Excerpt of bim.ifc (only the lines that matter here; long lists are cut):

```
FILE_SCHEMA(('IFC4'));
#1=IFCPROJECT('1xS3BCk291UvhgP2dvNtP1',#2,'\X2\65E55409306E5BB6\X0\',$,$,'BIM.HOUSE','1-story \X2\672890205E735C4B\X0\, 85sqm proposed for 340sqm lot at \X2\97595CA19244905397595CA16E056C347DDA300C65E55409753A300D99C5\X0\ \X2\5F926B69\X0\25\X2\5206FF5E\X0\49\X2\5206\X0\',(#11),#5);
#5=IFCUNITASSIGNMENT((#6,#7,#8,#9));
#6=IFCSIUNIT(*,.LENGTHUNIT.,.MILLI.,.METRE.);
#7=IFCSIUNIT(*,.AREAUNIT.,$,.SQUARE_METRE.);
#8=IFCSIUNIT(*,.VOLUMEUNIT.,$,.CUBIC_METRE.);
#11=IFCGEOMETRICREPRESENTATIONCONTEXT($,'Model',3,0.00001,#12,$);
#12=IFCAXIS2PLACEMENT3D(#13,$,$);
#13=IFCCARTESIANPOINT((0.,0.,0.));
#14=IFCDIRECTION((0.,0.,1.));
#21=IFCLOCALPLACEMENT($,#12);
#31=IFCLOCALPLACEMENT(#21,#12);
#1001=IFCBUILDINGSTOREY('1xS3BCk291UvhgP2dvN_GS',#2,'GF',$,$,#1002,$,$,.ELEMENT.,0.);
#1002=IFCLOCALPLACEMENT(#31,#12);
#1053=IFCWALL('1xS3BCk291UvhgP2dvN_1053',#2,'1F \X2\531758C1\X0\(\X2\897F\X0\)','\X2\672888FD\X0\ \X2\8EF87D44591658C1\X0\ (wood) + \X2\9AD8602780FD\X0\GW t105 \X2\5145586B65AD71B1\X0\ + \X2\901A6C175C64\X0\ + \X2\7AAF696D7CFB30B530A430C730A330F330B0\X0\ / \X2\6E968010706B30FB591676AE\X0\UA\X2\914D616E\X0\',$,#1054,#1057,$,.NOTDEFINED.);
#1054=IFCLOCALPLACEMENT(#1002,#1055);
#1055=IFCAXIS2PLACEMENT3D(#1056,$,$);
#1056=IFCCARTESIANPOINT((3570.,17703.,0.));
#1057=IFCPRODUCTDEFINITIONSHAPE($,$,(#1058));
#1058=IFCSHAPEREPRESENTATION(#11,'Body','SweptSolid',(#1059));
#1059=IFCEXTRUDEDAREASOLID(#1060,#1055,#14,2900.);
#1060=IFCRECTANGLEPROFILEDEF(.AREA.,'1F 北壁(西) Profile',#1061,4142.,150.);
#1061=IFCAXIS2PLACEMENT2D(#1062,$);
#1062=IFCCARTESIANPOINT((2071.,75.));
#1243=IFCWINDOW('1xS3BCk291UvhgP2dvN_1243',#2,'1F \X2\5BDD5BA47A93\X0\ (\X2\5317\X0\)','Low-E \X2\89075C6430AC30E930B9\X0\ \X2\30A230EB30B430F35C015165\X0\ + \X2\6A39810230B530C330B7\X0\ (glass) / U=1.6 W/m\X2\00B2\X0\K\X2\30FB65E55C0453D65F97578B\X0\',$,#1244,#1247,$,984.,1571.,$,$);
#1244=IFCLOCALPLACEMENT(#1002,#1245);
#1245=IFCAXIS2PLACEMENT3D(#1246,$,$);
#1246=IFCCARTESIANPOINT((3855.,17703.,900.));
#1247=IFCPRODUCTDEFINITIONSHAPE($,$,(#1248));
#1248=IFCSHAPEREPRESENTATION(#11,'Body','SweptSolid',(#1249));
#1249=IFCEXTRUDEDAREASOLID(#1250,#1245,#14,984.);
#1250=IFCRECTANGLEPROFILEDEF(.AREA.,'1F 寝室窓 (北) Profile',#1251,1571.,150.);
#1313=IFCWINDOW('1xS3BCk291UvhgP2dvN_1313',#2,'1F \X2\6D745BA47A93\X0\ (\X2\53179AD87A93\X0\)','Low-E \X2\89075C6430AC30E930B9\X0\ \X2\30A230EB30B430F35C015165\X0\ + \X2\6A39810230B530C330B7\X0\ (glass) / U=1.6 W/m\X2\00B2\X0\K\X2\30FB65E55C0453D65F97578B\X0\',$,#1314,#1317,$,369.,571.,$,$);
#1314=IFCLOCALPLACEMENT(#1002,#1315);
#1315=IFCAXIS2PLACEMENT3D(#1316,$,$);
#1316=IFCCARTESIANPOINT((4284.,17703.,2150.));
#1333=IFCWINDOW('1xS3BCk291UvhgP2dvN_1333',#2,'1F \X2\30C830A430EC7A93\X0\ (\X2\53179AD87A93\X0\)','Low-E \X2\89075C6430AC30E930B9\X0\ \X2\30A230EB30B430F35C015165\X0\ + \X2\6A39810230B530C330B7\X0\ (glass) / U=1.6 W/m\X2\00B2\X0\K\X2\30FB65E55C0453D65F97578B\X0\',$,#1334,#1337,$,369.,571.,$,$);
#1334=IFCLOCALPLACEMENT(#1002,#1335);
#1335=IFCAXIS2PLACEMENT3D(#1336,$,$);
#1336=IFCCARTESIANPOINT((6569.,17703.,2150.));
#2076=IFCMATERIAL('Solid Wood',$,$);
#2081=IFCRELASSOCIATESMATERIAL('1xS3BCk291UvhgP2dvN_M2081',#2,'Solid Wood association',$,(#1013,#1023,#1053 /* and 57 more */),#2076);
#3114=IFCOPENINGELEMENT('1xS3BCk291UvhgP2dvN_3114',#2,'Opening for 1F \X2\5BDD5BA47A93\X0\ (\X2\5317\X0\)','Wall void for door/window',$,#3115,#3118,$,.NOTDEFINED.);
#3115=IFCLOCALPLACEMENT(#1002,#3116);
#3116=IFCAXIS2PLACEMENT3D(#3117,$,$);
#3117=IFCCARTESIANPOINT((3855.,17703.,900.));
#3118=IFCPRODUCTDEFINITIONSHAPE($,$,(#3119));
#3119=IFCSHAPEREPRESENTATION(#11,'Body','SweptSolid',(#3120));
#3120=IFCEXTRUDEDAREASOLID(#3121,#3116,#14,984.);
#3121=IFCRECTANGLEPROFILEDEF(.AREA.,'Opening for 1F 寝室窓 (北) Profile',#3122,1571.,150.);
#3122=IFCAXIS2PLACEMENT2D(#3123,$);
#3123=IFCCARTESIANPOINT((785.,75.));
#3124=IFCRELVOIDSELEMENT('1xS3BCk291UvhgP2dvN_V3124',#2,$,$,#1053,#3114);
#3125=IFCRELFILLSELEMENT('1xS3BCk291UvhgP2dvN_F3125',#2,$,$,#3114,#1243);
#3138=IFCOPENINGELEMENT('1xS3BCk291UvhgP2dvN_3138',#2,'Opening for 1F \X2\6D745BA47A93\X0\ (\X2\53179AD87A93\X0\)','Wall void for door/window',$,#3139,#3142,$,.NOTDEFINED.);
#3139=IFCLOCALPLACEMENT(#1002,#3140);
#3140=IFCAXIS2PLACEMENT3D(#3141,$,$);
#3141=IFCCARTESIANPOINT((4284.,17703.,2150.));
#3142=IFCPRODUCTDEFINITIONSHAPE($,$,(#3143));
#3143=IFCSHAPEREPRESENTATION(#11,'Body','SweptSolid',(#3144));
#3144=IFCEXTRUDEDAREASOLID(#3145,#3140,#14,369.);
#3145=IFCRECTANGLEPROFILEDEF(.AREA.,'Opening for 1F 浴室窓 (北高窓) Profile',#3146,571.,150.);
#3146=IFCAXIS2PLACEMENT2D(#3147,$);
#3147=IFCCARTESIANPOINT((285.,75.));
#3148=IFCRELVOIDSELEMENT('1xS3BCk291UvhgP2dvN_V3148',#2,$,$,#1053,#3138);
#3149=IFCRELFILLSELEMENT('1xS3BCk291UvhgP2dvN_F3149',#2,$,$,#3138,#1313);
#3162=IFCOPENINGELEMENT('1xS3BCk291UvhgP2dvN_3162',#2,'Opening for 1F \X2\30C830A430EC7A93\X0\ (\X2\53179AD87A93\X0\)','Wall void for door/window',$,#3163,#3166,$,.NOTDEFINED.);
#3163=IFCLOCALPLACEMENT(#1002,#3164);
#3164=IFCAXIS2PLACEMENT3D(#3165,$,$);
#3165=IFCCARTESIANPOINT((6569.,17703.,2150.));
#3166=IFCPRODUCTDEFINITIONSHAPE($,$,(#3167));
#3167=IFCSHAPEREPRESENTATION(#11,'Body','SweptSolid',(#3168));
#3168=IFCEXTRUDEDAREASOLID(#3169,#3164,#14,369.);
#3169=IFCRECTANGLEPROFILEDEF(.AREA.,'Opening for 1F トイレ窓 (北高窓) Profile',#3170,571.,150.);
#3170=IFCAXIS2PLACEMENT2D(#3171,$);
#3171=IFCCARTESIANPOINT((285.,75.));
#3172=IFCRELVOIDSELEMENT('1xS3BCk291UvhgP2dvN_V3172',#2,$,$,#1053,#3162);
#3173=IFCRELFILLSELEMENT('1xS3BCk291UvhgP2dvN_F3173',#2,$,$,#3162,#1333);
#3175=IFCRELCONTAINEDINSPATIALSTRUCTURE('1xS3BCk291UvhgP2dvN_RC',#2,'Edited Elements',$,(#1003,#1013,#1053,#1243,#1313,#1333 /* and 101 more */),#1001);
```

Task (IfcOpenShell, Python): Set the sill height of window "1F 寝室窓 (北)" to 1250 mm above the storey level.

```python
import numpy as np
import ifcopenshell
import ifcopenshell.api.geometry
import ifcopenshell.geom
import ifcopenshell.util.element
import ifcopenshell.util.placement
import ifcopenshell.util.shape
import ifcopenshell.util.unit

model = ifcopenshell.open("bim.ifc")
unit_scale = ifcopenshell.util.unit.calculate_unit_scale(model)

window = model.by_guid("1xS3BCk291UvhgP2dvN_1243")
opening = window.FillsVoids[0].RelatingOpeningElement
storey = ifcopenshell.util.element.get_container(window, ifc_class="IfcBuildingStorey")
level = ifcopenshell.util.placement.get_local_placement(storey.ObjectPlacement)[2, 3]

# The opening's origin need not be at the sill, so measure its lowest point.
shape = ifcopenshell.geom.create_shape(ifcopenshell.geom.settings(), opening)
bottom = ifcopenshell.util.shape.get_shape_bottom_elevation(shape, shape.geometry) / unit_scale
dz = level + 1250.0 - bottom

shift = np.array([0.0, 0.0, dz])
# The window is not placed relative to its opening, so move both.
for product in (opening, window):
    matrix = ifcopenshell.util.placement.get_local_placement(product.ObjectPlacement)
    matrix[:3, 3] += shift
    ifcopenshell.api.geometry.edit_object_placement(model, product=product, matrix=matrix, is_si=False)

print(f"moved by {dz * unit_scale:+.3f} m")

model.write("bim-out.ifc")
```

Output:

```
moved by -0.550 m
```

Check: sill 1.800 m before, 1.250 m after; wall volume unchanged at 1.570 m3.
